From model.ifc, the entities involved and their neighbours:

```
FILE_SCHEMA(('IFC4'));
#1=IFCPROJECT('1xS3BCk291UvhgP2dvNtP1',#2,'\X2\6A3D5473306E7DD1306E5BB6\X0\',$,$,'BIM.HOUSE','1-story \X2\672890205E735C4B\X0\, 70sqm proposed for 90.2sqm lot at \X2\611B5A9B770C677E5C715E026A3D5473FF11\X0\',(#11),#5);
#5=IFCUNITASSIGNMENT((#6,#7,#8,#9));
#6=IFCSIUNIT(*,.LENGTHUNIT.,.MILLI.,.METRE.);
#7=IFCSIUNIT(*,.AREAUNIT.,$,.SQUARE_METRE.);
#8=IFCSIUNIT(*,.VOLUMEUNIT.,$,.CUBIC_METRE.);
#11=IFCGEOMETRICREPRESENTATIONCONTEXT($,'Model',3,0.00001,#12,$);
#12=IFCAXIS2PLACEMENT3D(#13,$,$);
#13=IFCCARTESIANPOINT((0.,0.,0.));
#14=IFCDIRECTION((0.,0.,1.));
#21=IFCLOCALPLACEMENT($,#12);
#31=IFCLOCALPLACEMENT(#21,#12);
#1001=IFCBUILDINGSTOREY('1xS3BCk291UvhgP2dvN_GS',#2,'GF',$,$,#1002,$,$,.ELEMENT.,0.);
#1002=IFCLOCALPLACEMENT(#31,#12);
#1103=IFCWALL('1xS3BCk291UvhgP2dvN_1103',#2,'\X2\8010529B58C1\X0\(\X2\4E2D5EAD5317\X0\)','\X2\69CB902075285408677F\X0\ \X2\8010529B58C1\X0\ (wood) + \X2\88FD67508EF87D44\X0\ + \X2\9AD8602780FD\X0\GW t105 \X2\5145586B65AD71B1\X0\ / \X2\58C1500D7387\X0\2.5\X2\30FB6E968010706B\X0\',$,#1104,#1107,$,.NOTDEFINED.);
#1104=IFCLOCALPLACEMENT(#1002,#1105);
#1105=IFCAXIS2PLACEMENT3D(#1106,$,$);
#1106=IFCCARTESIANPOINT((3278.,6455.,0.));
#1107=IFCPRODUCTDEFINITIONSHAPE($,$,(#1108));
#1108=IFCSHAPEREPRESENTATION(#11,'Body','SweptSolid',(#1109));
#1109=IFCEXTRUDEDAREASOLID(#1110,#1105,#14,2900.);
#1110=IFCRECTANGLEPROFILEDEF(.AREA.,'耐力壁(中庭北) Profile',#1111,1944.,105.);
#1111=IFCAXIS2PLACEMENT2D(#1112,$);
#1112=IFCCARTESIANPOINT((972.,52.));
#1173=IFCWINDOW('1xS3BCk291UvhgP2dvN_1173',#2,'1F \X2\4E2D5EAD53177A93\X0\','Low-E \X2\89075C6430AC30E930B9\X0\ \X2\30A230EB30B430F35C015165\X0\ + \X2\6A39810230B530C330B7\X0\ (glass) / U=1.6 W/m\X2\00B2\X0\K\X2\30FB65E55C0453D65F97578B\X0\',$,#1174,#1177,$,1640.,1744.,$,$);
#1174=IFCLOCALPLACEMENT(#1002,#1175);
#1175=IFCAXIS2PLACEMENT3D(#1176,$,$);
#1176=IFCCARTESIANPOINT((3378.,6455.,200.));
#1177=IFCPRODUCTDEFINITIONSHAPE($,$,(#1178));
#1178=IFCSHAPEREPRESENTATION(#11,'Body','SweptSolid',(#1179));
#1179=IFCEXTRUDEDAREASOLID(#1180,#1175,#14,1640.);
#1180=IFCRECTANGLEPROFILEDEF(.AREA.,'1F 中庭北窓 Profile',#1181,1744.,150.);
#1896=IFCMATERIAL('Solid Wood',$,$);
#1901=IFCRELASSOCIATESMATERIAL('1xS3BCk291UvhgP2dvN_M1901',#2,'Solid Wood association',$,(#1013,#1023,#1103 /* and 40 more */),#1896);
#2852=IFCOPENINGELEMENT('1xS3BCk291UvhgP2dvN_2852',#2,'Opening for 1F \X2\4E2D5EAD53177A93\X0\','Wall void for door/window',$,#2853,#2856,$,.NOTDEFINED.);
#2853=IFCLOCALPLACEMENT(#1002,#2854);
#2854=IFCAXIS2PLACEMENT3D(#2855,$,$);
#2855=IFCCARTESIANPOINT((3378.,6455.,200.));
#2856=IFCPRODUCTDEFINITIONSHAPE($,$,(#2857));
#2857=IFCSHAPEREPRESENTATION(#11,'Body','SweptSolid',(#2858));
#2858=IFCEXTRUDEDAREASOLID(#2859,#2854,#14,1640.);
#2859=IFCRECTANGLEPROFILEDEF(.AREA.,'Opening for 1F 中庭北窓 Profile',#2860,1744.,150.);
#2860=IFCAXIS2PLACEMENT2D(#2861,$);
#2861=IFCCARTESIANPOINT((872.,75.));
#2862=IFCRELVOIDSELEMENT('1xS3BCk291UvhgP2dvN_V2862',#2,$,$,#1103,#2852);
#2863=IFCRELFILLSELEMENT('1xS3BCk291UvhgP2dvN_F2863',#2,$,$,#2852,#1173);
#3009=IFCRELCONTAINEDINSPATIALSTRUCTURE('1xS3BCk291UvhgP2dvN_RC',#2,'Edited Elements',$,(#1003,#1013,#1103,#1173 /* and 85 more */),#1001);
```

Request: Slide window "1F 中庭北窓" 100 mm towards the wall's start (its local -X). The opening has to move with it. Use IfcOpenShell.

```python
import ifcopenshell
import ifcopenshell.api.geometry
import ifcopenshell.util.placement

model = ifcopenshell.open("model.ifc")

window = model.by_guid("1xS3BCk291UvhgP2dvN_1173")
opening = window.FillsVoids[0].RelatingOpeningElement
wall = opening.VoidsElements[0].RelatingBuildingElement

wall_matrix = ifcopenshell.util.placement.get_local_placement(wall.ObjectPlacement)
shift = wall_matrix[:3, 0] * -100.0
before = ifcopenshell.util.placement.get_local_placement(window.ObjectPlacement)[:3, 3].copy()

# The window is not placed relative to its opening, so move both.
for product in (opening, window):
    matrix = ifcopenshell.util.placement.get_local_placement(product.ObjectPlacement)
    matrix[:3, 3] += shift
    ifcopenshell.api.geometry.edit_object_placement(model, product=product, matrix=matrix, is_si=False)

after = ifcopenshell.util.placement.get_local_placement(window.ObjectPlacement)[:3, 3]
print("window moved by", (after - before).round(3) + 0.0)

model.write("model_rev.ifc")
```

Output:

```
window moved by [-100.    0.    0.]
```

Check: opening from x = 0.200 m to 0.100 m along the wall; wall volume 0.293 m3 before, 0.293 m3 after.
